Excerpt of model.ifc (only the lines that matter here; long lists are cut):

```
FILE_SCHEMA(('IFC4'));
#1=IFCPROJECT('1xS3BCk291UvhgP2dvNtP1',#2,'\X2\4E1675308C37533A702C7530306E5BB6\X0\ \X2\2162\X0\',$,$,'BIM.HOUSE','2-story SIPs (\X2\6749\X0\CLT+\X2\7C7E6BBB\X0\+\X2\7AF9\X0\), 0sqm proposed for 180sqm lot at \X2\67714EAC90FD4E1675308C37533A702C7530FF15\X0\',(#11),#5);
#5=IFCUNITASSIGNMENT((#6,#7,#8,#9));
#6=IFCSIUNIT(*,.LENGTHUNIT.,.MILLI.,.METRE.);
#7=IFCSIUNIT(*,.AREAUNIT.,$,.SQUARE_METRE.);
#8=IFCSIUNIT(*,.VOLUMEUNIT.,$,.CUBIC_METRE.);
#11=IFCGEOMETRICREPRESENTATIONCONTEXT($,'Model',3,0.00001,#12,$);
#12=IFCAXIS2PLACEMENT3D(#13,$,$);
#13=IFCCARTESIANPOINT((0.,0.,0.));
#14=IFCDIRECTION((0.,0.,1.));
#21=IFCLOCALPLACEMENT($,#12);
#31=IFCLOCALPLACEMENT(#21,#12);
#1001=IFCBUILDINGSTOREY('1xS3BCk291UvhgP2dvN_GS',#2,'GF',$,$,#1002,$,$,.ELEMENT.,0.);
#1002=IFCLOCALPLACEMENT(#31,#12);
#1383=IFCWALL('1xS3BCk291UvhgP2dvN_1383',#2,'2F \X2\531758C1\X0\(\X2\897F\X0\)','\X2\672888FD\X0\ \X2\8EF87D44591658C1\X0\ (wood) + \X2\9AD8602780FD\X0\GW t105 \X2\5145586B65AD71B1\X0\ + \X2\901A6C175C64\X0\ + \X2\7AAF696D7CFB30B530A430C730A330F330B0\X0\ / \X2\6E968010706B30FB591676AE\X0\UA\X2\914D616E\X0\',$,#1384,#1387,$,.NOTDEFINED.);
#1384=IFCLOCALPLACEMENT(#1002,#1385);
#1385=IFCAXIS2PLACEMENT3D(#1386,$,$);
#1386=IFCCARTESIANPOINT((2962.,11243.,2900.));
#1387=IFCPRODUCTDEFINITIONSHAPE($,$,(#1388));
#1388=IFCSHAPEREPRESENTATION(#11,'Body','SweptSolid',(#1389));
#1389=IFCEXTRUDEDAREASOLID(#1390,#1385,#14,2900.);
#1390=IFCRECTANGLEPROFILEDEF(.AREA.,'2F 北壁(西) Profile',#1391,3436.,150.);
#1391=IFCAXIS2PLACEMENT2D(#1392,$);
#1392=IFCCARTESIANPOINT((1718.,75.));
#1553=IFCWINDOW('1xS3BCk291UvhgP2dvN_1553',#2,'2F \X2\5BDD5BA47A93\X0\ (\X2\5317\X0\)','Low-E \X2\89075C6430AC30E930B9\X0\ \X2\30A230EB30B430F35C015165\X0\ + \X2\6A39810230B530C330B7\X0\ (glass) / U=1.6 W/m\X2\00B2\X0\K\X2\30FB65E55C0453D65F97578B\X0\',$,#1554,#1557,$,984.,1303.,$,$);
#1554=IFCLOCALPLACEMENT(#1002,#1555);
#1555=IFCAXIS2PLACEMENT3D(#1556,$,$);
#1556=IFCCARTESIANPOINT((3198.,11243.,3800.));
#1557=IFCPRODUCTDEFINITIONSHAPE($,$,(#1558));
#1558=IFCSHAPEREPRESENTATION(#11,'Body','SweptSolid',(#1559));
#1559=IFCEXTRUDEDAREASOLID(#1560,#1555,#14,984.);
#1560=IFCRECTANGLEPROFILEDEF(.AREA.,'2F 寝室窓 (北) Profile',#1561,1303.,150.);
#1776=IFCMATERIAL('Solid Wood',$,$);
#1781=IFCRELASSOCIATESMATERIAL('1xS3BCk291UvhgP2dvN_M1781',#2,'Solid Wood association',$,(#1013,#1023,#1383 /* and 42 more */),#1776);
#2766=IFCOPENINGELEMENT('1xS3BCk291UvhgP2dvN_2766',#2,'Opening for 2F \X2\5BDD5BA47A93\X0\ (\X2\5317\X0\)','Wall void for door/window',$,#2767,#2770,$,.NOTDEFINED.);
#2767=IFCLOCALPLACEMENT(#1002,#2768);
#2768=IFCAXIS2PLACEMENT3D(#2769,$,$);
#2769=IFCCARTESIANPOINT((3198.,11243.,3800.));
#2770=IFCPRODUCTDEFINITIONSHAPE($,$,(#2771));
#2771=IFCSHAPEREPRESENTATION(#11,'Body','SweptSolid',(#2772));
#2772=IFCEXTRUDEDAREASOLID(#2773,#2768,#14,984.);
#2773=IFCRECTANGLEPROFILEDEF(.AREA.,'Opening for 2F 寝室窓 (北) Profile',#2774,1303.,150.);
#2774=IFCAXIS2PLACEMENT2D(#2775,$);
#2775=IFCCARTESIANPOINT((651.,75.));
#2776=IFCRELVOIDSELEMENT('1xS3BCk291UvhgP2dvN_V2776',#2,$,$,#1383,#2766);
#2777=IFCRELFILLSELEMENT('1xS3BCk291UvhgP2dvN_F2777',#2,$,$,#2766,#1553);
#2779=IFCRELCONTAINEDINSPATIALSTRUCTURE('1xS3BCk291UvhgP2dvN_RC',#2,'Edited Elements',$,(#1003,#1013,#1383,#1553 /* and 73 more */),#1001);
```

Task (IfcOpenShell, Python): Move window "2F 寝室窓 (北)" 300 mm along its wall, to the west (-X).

```python
import ifcopenshell
import ifcopenshell.api.geometry
import ifcopenshell.util.placement

model = ifcopenshell.open("model.ifc")

window = model.by_id(1553)
opening = window.FillsVoids[0].RelatingOpeningElement
wall = opening.VoidsElements[0].RelatingBuildingElement

wall_matrix = ifcopenshell.util.placement.get_local_placement(wall.ObjectPlacement)
shift = wall_matrix[:3, 0] * -300.0
before = ifcopenshell.util.placement.get_local_placement(window.ObjectPlacement)[:3, 3].copy()

# The window is not placed relative to its opening, so move both.
for product in (opening, window):
    matrix = ifcopenshell.util.placement.get_local_placement(product.ObjectPlacement)
    matrix[:3, 3] += shift
    ifcopenshell.api.geometry.edit_object_placement(model, product=product, matrix=matrix, is_si=False)

after = ifcopenshell.util.placement.get_local_placement(window.ObjectPlacement)[:3, 3]
print("window moved by", (after - before).round(3) + 0.0)

model.write("model-out.ifc")
```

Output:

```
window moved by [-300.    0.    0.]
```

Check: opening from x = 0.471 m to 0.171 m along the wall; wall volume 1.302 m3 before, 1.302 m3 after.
